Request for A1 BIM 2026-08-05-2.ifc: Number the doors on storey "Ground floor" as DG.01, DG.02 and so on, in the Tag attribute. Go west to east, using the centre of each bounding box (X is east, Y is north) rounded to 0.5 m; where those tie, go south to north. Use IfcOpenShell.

First a look at what the model holds.

```python
import ifcopenshell
import ifcopenshell.util.element
import ifcopenshell.util.placement

model = ifcopenshell.open("A1 BIM 2026-08-05-2.ifc")
print(model.schema)
storey = next(s for s in model.by_type("IfcBuildingStorey") if s.Name == "Ground floor")
doors = [e for e in ifcopenshell.util.element.get_decomposition(storey) if e.is_a("IfcDoor")]
for e in sorted(doors, key=lambda e: e.id()):
    origin = ifcopenshell.util.placement.get_local_placement(e.ObjectPlacement)[:3, 3]
    print(e.id(), e.Tag, e.Name, origin.round(2) + 0.0, sep=" | ")
```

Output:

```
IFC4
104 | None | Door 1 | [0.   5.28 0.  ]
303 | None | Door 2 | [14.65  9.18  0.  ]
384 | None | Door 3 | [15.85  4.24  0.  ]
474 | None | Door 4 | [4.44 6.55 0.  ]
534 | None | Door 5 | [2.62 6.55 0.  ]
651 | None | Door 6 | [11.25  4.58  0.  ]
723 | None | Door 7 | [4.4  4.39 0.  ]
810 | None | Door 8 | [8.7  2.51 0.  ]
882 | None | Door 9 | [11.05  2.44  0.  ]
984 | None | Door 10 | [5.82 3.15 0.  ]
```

```python
import ifcopenshell
import ifcopenshell.geom
import ifcopenshell.util.element
import ifcopenshell.util.shape

model = ifcopenshell.open("A1 BIM 2026-08-05-2.ifc")
settings = ifcopenshell.geom.settings()
settings.set("use-world-coords", True)


def centre(element):
    shape = ifcopenshell.geom.create_shape(settings, element)
    return ifcopenshell.util.shape.get_bbox_centroid(shape.geometry)


storey = next(s for s in model.by_type("IfcBuildingStorey") if s.Name == "Ground floor")
doors = [e for e in ifcopenshell.util.element.get_decomposition(storey) if e.is_a("IfcDoor")]

# Insertion points can sit at a corner or the storey origin, so sort by the geometry (in metres).
centres = {e: centre(e) for e in doors}
doors.sort(key=lambda e: (round(centres[e][0] / 0.5), centres[e][1]))

for i, e in enumerate(doors, start=1):
    number = f"DG.{i:02d}"
    e.Tag = number
    print(e.id(), number)

model.write("A1 BIM 2026-08-05-2_updated.ifc")
```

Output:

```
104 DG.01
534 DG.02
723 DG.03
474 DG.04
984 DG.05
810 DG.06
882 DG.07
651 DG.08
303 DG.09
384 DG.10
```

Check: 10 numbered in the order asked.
